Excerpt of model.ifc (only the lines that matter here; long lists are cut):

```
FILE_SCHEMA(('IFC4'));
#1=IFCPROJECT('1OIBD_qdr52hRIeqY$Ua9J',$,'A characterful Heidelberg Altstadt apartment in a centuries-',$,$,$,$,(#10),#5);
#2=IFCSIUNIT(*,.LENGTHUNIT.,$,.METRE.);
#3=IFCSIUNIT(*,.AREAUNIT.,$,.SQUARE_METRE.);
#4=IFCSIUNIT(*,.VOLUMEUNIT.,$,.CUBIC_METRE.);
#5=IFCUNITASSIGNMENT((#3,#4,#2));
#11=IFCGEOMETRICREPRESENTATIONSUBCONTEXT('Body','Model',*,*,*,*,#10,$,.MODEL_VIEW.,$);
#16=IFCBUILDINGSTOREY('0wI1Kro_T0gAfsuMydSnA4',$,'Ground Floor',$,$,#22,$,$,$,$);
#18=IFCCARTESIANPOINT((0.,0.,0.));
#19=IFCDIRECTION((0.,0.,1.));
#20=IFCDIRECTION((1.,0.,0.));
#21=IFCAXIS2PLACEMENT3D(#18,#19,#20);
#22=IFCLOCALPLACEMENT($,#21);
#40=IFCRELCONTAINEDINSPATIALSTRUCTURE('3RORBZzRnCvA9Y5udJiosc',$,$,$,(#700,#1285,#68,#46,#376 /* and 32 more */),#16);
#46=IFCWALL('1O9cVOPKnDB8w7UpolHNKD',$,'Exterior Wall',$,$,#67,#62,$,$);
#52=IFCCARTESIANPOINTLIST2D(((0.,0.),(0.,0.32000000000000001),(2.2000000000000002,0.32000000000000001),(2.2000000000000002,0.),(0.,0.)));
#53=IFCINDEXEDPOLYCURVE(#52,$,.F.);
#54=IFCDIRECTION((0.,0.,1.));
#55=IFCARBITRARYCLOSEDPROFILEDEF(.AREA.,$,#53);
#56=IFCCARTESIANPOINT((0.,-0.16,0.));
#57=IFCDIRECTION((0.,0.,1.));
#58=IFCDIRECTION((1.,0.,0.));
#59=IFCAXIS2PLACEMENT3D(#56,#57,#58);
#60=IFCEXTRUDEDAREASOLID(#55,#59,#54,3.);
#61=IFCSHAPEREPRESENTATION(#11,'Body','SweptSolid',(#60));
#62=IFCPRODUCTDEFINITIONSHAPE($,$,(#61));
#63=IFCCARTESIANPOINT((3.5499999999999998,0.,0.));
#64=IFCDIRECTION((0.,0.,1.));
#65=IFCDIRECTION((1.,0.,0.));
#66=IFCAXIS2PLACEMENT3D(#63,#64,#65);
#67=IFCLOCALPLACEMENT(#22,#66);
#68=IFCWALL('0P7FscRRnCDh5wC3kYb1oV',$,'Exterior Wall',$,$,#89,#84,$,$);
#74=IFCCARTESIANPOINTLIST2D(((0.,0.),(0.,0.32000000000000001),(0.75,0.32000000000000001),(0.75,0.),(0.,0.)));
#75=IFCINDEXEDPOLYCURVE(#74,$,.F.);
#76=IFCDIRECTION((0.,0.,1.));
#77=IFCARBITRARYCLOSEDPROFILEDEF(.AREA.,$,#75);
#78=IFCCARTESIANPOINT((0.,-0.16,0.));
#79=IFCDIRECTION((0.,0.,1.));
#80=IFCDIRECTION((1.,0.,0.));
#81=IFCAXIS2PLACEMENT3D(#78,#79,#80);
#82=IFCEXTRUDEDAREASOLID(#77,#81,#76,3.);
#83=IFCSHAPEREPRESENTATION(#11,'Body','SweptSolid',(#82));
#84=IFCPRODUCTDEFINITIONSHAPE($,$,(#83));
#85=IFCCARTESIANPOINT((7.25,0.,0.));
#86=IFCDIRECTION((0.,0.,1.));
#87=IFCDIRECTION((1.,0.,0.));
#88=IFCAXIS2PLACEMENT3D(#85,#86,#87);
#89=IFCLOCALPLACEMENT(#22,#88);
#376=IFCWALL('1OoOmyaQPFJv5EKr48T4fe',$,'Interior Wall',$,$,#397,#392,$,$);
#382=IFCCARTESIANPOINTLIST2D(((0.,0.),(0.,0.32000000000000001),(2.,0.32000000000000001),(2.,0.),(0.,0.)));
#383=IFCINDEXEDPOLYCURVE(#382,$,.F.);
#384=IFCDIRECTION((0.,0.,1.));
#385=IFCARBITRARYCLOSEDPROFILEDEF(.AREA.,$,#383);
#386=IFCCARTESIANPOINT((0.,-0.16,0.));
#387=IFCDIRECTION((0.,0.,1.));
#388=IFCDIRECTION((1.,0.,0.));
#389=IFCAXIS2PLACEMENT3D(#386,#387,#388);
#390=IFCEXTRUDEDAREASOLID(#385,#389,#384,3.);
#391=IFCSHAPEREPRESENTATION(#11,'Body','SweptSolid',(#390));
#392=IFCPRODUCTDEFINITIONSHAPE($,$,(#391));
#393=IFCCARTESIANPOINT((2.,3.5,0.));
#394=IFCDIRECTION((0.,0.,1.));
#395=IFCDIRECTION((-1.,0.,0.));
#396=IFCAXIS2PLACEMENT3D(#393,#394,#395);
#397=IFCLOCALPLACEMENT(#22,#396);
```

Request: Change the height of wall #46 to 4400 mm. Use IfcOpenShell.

```python
import ifcopenshell
import ifcopenshell.geom
import ifcopenshell.util.representation
import ifcopenshell.util.shape
import ifcopenshell.util.unit

model = ifcopenshell.open("model.ifc")
unit_scale = ifcopenshell.util.unit.calculate_unit_scale(model)
settings = ifcopenshell.geom.settings()


def volume(element):
    """Net volume in cubic metres, openings subtracted."""
    shape = ifcopenshell.geom.create_shape(settings, element)
    return ifcopenshell.util.shape.get_volume(shape.geometry)


wall = model.by_id(46)
before = volume(wall)

body = ifcopenshell.util.representation.get_representation(wall, "Model", "Body")
solid = body.Items[0]
old_height = solid.Depth
solid.Depth = 4.4 / unit_scale
after = volume(wall)

print(f"height {old_height:g} -> {solid.Depth:g}, volume {before:.3f} -> {after:.3f} m3")

model.write("model_v2.ifc")
```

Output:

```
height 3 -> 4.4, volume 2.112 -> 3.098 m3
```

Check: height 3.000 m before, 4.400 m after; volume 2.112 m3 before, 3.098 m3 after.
